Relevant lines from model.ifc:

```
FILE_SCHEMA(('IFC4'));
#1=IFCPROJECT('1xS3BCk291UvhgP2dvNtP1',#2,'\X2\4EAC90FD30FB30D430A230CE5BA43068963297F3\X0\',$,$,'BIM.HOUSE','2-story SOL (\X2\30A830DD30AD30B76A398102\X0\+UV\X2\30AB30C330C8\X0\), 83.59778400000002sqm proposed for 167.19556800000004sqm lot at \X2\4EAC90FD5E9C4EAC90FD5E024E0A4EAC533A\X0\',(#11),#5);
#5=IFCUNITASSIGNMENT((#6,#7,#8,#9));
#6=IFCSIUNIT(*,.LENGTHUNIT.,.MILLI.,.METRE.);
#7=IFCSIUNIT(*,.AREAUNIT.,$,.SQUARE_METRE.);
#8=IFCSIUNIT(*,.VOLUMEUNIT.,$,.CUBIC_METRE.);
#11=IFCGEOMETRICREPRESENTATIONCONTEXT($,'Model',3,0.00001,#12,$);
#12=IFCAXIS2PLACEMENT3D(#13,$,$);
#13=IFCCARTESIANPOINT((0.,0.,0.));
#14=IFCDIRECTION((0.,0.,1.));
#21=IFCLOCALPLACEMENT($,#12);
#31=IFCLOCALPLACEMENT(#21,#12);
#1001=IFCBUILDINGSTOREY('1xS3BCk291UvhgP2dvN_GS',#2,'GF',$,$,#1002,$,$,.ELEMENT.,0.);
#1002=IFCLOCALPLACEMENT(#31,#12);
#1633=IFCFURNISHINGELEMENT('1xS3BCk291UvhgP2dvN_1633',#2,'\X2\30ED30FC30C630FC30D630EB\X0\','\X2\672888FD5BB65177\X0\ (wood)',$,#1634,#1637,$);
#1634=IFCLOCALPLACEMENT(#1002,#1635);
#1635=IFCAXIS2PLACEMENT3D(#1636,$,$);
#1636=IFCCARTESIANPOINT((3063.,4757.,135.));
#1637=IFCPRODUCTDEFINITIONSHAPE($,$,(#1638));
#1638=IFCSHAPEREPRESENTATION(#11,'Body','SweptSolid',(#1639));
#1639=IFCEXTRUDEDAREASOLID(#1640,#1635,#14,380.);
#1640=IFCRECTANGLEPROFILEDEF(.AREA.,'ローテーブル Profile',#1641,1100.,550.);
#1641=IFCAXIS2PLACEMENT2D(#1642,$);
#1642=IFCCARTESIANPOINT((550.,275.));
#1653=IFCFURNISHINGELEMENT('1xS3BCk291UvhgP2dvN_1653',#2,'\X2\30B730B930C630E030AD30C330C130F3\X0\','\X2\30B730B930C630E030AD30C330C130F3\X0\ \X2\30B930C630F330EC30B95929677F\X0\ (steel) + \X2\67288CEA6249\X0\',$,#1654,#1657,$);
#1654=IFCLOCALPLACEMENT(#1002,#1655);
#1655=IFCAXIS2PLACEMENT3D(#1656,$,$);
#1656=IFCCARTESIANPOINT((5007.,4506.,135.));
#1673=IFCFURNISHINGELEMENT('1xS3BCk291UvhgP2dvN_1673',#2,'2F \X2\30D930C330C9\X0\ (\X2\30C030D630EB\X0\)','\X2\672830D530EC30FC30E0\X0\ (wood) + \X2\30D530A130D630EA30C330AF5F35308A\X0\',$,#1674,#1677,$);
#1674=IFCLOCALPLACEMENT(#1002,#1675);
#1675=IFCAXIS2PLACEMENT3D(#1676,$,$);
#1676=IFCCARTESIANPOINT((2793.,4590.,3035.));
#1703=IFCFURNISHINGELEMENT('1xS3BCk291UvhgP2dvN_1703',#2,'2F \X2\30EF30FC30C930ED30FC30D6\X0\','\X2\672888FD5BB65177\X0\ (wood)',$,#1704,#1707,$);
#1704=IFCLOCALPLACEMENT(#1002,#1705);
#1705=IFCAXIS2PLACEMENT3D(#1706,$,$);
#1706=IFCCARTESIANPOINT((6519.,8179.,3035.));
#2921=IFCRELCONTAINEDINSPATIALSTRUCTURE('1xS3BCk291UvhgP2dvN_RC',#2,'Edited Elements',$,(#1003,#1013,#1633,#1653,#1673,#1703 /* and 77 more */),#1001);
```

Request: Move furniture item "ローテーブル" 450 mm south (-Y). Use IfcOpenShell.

```python
import ifcopenshell
import ifcopenshell.api.geometry
import ifcopenshell.util.placement
import ifcopenshell.util.unit

model = ifcopenshell.open("model.ifc")
unit_scale = ifcopenshell.util.unit.calculate_unit_scale(model)

item = model.by_id(1633)
matrix = ifcopenshell.util.placement.get_local_placement(item.ObjectPlacement)
matrix[1, 3] -= 0.45 / unit_scale
ifcopenshell.api.geometry.edit_object_placement(model, product=item, matrix=matrix, is_si=False)

print(ifcopenshell.util.placement.get_local_placement(item.ObjectPlacement).round(3) + 0.0)

model.write("model_edited.ifc")
```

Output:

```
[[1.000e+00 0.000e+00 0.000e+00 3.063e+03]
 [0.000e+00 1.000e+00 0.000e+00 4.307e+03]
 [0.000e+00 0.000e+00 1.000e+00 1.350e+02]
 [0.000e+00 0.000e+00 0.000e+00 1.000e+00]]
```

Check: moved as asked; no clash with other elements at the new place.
